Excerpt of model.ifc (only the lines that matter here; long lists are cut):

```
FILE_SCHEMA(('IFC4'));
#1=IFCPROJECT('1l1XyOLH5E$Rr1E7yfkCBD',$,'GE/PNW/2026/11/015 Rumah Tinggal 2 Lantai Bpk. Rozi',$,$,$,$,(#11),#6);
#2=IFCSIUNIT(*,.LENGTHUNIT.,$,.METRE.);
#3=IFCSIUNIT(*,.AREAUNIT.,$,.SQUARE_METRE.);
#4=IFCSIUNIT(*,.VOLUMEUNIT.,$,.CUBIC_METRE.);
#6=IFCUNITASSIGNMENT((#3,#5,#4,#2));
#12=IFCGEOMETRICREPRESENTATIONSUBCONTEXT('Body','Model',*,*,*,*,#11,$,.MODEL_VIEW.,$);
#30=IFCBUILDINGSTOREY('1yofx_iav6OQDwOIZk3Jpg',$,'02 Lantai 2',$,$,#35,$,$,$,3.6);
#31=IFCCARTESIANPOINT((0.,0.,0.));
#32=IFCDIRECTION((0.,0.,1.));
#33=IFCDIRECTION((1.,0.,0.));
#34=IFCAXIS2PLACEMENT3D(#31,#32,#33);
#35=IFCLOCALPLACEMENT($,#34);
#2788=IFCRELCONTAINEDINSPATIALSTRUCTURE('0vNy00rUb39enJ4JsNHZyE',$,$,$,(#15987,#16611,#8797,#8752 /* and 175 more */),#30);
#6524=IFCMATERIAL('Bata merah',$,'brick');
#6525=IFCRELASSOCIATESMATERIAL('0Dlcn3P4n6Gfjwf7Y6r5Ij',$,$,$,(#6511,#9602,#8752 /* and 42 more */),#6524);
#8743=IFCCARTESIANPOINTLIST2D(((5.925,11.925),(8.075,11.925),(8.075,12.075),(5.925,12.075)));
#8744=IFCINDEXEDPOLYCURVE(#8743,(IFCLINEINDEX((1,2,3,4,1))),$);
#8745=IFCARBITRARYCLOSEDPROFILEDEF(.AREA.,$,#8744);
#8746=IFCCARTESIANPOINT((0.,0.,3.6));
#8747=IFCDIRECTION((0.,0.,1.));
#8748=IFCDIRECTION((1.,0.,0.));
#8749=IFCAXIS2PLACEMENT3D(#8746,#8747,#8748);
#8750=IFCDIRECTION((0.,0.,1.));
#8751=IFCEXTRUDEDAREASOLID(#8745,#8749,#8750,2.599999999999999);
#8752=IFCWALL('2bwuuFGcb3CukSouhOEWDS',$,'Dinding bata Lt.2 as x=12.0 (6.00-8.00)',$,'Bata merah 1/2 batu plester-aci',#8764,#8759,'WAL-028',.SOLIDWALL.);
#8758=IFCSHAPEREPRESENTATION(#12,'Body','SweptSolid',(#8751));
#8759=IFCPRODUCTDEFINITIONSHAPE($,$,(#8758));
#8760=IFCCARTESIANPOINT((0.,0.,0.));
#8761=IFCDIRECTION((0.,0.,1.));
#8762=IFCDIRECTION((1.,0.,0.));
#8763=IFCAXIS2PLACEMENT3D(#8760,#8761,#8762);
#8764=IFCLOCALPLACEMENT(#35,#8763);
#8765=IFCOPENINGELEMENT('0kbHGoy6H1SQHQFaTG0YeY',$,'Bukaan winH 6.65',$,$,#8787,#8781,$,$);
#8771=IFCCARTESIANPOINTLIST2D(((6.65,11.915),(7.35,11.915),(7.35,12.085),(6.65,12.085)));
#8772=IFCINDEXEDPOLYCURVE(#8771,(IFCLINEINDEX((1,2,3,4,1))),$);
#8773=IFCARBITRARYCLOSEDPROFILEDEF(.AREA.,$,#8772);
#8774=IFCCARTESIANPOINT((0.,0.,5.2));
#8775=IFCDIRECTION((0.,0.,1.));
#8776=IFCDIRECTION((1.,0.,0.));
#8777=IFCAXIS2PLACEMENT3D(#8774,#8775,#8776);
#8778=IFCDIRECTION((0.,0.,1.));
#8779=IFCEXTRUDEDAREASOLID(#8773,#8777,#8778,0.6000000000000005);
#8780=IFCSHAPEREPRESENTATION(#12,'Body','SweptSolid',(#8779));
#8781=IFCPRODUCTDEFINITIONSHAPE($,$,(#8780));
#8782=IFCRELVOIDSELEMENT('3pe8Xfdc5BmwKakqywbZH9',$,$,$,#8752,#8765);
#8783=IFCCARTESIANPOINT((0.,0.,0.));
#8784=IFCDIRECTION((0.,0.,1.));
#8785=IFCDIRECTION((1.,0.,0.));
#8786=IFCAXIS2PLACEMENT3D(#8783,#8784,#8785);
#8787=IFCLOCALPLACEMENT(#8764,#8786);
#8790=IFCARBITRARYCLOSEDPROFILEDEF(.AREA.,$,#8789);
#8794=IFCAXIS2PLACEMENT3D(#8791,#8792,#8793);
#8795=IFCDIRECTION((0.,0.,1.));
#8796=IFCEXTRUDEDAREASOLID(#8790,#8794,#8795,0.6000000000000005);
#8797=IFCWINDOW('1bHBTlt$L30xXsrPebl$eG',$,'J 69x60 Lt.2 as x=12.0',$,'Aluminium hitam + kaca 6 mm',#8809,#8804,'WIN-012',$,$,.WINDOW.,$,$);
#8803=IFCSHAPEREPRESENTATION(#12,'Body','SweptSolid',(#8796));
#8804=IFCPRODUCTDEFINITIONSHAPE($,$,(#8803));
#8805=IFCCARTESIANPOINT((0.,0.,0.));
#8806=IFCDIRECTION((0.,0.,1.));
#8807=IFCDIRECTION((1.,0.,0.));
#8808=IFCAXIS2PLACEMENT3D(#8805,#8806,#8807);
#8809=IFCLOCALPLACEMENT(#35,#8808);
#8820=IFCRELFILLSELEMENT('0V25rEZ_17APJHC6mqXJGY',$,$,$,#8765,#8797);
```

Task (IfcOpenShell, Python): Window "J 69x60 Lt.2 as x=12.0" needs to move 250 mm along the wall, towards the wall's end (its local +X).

```python
import ifcopenshell
import ifcopenshell.api.geometry
import ifcopenshell.util.placement
import ifcopenshell.util.unit

model = ifcopenshell.open("model.ifc")
unit_scale = ifcopenshell.util.unit.calculate_unit_scale(model)

window = model.by_id(8797)
opening = window.FillsVoids[0].RelatingOpeningElement
wall = opening.VoidsElements[0].RelatingBuildingElement

wall_matrix = ifcopenshell.util.placement.get_local_placement(wall.ObjectPlacement)
shift = wall_matrix[:3, 0] * 0.25 / unit_scale
before = ifcopenshell.util.placement.get_local_placement(window.ObjectPlacement)[:3, 3].copy()

# The window is not placed relative to its opening, so move both.
for product in (opening, window):
    matrix = ifcopenshell.util.placement.get_local_placement(product.ObjectPlacement)
    matrix[:3, 3] += shift
    ifcopenshell.api.geometry.edit_object_placement(model, product=product, matrix=matrix, is_si=False)

after = ifcopenshell.util.placement.get_local_placement(window.ObjectPlacement)[:3, 3]
print("window moved by", (after - before).round(3) + 0.0)

model.write("model_edited.ifc")
```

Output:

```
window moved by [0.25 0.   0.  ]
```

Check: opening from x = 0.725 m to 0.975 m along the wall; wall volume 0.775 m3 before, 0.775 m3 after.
